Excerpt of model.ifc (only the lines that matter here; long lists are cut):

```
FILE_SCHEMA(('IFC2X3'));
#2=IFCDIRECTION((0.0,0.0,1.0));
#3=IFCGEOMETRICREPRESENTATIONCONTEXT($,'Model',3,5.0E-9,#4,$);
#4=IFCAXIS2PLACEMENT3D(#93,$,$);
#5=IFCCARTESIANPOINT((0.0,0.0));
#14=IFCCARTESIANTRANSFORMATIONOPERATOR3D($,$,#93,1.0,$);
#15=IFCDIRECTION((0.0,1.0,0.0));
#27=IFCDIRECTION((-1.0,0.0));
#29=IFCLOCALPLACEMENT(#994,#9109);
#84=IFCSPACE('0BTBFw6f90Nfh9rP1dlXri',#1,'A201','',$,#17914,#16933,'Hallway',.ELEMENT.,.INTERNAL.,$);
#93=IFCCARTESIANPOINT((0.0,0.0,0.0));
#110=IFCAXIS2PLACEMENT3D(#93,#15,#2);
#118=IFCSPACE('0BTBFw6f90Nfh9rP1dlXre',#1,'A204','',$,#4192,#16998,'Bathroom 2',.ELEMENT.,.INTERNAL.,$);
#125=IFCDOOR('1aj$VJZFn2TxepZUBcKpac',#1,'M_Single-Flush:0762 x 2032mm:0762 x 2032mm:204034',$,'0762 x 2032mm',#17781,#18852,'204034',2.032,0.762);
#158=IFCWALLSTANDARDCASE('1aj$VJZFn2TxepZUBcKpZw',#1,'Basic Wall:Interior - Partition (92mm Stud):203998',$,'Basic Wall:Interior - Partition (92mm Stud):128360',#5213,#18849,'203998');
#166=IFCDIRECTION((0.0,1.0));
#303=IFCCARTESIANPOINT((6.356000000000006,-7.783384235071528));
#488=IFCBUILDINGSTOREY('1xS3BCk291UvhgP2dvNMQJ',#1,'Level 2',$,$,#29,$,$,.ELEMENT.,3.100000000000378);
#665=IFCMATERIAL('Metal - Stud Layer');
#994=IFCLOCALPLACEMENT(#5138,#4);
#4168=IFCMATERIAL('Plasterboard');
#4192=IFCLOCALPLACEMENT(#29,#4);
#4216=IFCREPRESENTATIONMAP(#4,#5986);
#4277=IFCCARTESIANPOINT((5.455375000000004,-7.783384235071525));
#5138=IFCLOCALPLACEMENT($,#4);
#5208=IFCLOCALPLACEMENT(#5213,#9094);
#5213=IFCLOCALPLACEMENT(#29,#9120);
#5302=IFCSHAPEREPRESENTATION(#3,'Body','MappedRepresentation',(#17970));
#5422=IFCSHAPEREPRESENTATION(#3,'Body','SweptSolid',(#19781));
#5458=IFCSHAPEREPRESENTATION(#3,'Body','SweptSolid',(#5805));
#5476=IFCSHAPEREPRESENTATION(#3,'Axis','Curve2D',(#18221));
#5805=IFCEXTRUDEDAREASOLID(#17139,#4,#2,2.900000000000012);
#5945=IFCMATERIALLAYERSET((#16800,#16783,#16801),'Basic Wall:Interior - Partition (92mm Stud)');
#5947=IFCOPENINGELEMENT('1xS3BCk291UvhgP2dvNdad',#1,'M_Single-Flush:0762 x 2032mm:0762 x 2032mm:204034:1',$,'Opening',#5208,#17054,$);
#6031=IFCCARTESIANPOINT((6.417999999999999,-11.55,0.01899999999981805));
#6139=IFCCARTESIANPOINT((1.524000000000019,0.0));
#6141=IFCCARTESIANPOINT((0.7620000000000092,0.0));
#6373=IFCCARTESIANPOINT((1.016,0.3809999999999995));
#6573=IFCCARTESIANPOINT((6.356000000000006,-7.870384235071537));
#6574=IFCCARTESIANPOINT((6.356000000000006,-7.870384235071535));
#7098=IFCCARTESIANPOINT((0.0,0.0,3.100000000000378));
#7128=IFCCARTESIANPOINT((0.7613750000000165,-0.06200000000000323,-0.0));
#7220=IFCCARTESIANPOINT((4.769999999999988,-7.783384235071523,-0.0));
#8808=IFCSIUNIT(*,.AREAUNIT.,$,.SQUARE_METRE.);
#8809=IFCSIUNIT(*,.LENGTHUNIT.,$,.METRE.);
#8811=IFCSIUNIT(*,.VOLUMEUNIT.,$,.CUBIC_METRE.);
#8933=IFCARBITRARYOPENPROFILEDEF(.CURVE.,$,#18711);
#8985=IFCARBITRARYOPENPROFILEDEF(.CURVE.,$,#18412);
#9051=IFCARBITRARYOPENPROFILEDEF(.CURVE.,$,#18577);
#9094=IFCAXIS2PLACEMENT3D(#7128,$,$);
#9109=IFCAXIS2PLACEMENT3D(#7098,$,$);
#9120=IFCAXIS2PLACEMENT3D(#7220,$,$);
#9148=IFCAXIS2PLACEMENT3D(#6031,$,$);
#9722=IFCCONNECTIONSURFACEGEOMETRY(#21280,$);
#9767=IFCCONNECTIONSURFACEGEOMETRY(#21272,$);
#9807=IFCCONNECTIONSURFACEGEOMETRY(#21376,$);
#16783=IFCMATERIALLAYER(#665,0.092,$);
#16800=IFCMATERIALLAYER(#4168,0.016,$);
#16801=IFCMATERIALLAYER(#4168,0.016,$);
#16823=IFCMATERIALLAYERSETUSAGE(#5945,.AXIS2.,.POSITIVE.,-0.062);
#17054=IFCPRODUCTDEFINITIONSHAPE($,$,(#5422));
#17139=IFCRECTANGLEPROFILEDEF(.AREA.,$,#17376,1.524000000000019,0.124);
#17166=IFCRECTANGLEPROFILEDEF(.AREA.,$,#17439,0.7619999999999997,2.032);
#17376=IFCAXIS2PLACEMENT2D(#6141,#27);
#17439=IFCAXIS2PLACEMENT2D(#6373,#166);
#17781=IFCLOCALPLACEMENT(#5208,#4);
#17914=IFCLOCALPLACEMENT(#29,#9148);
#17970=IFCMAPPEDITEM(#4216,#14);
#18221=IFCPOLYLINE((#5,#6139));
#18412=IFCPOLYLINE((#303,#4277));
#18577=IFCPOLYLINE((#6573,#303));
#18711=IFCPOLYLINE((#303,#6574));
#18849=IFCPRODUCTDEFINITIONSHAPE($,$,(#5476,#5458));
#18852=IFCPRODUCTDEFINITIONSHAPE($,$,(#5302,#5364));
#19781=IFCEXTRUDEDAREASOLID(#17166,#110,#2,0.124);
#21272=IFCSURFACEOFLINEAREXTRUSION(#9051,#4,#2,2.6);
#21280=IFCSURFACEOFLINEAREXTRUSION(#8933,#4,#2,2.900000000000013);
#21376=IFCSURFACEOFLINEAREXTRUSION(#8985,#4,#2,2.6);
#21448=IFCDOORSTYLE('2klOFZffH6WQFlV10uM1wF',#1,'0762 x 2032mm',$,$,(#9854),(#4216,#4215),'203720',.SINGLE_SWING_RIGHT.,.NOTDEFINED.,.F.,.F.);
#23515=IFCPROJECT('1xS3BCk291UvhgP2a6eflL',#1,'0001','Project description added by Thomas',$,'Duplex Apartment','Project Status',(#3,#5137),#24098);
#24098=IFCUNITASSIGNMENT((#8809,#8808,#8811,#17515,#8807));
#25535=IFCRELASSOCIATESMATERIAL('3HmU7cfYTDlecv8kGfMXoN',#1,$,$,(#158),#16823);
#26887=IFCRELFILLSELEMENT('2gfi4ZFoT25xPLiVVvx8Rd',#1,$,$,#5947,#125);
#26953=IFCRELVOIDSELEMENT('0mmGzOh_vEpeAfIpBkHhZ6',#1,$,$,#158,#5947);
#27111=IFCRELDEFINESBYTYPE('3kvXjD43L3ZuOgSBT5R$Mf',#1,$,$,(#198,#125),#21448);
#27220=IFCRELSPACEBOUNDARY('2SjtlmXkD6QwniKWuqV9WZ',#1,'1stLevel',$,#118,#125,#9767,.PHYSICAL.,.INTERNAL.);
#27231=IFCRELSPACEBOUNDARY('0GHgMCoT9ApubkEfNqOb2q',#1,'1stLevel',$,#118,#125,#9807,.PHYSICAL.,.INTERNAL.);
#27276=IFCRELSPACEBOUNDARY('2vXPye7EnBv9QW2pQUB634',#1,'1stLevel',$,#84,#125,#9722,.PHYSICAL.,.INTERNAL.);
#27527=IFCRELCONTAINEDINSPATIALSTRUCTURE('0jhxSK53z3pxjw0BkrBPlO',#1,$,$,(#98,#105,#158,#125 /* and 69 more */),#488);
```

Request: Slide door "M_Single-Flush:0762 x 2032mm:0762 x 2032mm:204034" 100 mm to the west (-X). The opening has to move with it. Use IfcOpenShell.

```python
import numpy as np
import ifcopenshell
import ifcopenshell.api.geometry
import ifcopenshell.util.placement
import ifcopenshell.util.unit

model = ifcopenshell.open("model.ifc")
unit_scale = ifcopenshell.util.unit.calculate_unit_scale(model)

door = model.by_id(125)
opening = door.FillsVoids[0].RelatingOpeningElement
wall = opening.VoidsElements[0].RelatingBuildingElement

wall_matrix = ifcopenshell.util.placement.get_local_placement(wall.ObjectPlacement)
shift = wall_matrix[:3, 0] * -0.1 / unit_scale
before = ifcopenshell.util.placement.get_local_placement(door.ObjectPlacement)[:3, 3].copy()

# The door is placed relative to its opening, so it follows when the opening moves.
matrix = ifcopenshell.util.placement.get_local_placement(opening.ObjectPlacement)
matrix[:3, 3] += shift
ifcopenshell.api.geometry.edit_object_placement(
    model, product=opening, matrix=matrix, is_si=False, should_transform_children=True
)

# Space boundary surfaces are stored in each space's coordinates; move them too.
for rel in door.ProvidesBoundaries:
    if not rel.ConnectionGeometry:
        continue
    surface = rel.ConnectionGeometry.SurfaceOnRelatingElement
    space_matrix = ifcopenshell.util.placement.get_local_placement(rel.RelatingSpace.ObjectPlacement)
    point = np.array(surface.Position.Location.Coordinates) + space_matrix[:3, :3].T @ shift
    surface.Position = model.createIfcAxis2Placement3D(
        model.createIfcCartesianPoint(point.tolist()), surface.Position.Axis, surface.Position.RefDirection
    )

after = ifcopenshell.util.placement.get_local_placement(door.ObjectPlacement)[:3, 3]
print("door moved by", (after - before).round(3) + 0.0)

model.write("model_rev.ifc")
```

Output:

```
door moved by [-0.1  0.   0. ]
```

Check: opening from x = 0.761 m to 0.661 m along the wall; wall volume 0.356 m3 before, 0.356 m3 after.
